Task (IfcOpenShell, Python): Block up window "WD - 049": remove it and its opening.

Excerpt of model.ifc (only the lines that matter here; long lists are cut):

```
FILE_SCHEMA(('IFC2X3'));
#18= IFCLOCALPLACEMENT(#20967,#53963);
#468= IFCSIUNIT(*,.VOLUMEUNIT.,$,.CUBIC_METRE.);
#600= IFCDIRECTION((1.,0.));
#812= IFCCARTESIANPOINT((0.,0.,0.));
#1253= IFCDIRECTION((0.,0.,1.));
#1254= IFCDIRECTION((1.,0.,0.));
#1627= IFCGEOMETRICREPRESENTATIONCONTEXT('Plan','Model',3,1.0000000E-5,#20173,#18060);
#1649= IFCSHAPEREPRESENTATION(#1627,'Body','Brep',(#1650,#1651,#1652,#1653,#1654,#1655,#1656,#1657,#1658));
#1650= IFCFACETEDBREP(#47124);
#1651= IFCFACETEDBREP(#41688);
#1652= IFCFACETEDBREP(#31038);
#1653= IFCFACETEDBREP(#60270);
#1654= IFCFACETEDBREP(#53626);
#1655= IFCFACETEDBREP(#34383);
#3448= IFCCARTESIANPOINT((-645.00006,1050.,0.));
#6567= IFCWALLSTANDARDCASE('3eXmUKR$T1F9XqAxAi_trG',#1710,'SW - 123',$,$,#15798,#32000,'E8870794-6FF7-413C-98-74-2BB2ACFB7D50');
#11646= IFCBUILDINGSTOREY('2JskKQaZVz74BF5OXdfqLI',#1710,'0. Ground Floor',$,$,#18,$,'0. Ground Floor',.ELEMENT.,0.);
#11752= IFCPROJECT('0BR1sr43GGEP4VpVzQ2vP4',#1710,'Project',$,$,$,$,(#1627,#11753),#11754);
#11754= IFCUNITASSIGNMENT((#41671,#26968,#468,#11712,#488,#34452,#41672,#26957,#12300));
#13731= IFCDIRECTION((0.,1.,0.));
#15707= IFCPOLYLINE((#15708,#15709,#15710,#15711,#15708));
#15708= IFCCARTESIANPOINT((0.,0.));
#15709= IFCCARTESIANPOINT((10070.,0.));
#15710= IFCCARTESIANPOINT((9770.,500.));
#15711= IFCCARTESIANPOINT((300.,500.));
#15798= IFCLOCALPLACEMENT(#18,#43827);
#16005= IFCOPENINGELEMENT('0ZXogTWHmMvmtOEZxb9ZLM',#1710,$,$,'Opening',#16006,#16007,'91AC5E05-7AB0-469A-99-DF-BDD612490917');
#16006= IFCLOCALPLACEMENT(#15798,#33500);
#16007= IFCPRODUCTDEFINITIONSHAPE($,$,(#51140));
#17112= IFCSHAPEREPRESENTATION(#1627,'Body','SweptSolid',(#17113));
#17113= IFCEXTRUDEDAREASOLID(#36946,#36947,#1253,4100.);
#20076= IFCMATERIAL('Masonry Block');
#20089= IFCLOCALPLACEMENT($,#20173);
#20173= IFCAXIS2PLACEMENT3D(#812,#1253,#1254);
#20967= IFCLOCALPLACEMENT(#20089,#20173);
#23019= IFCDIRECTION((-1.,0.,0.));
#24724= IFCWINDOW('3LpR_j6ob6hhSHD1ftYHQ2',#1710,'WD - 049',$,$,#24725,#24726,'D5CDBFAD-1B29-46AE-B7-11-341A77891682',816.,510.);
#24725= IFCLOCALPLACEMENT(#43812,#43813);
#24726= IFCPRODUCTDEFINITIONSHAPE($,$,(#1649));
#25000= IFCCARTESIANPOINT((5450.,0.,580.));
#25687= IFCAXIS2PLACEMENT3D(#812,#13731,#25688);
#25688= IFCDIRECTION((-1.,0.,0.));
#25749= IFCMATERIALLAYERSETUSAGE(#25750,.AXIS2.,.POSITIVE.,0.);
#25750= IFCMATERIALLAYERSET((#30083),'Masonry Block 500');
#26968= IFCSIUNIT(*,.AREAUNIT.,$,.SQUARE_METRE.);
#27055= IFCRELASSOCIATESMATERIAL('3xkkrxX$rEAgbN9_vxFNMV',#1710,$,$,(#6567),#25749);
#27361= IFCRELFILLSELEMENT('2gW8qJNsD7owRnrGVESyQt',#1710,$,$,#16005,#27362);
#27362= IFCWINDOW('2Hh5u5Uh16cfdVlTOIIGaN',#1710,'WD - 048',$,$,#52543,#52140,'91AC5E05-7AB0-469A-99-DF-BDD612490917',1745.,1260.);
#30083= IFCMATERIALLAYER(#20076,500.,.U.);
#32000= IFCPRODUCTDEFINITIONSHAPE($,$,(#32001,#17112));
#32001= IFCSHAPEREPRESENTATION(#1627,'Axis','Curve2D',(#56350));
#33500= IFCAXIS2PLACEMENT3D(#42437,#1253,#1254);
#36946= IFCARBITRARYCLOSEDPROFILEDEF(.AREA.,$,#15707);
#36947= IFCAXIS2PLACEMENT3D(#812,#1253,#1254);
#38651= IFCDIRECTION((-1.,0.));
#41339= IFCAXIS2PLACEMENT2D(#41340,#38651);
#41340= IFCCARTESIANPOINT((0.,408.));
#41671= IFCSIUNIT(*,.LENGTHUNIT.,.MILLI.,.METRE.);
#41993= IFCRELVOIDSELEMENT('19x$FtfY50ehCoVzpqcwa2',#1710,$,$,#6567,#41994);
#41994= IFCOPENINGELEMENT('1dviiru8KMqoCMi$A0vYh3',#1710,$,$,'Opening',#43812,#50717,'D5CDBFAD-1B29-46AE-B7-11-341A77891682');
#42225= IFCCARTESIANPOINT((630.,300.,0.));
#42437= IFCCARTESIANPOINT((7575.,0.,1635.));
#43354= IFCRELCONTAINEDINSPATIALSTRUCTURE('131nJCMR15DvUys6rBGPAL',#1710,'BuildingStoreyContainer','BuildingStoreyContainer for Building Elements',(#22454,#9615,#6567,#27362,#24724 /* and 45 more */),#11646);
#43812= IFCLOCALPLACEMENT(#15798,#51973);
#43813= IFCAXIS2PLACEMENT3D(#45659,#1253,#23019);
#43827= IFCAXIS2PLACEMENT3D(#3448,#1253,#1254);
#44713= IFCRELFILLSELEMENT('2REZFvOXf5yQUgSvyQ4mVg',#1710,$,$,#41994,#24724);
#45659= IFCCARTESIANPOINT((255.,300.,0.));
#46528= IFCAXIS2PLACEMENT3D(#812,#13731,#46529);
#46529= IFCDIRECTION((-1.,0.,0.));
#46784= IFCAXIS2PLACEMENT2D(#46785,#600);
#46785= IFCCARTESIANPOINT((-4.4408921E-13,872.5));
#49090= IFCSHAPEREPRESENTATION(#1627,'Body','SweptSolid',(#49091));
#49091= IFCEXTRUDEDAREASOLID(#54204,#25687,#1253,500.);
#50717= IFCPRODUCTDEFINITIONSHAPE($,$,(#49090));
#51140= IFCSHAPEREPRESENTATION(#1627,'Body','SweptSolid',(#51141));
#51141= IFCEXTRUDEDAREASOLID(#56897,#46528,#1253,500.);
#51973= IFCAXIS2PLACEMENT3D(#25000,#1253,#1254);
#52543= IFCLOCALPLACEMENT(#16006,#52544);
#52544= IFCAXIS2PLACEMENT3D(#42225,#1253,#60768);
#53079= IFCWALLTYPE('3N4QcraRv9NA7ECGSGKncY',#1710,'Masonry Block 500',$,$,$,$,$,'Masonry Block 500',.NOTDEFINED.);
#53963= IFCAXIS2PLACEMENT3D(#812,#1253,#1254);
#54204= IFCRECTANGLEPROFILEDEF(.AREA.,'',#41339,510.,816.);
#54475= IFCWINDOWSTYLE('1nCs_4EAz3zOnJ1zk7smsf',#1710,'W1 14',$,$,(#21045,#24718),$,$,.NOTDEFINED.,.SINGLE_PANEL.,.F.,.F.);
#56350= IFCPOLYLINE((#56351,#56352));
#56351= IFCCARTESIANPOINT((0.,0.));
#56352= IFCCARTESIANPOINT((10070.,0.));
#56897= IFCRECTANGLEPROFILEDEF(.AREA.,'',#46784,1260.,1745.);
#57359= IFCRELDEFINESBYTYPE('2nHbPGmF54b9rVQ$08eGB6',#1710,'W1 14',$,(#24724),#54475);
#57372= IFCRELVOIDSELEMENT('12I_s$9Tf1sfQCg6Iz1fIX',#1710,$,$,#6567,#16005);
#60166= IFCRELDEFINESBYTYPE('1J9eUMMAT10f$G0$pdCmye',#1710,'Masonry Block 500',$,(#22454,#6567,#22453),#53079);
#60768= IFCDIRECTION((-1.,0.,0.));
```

```python
import ifcopenshell
import ifcopenshell.api.feature
import ifcopenshell.api.root
import ifcopenshell.geom
import ifcopenshell.util.shape

model = ifcopenshell.open("model.ifc")
settings = ifcopenshell.geom.settings()


def volume(element):
    """Net volume in cubic metres, openings subtracted."""
    shape = ifcopenshell.geom.create_shape(settings, element)
    return ifcopenshell.util.shape.get_volume(shape.geometry)


window = model.by_guid("3LpR_j6ob6hhSHD1ftYHQ2")
opening = window.FillsVoids[0].RelatingOpeningElement
wall = opening.VoidsElements[0].RelatingBuildingElement
before = volume(wall)

ifcopenshell.api.root.remove_product(model, product=window)
ifcopenshell.api.feature.remove_feature(model, feature=opening)

after = volume(wall)

print(f"wall volume {before:.3f} -> {after:.3f} m3")

model.write("model_rev.ifc")
```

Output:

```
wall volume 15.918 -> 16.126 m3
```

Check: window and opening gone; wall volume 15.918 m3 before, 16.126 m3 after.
